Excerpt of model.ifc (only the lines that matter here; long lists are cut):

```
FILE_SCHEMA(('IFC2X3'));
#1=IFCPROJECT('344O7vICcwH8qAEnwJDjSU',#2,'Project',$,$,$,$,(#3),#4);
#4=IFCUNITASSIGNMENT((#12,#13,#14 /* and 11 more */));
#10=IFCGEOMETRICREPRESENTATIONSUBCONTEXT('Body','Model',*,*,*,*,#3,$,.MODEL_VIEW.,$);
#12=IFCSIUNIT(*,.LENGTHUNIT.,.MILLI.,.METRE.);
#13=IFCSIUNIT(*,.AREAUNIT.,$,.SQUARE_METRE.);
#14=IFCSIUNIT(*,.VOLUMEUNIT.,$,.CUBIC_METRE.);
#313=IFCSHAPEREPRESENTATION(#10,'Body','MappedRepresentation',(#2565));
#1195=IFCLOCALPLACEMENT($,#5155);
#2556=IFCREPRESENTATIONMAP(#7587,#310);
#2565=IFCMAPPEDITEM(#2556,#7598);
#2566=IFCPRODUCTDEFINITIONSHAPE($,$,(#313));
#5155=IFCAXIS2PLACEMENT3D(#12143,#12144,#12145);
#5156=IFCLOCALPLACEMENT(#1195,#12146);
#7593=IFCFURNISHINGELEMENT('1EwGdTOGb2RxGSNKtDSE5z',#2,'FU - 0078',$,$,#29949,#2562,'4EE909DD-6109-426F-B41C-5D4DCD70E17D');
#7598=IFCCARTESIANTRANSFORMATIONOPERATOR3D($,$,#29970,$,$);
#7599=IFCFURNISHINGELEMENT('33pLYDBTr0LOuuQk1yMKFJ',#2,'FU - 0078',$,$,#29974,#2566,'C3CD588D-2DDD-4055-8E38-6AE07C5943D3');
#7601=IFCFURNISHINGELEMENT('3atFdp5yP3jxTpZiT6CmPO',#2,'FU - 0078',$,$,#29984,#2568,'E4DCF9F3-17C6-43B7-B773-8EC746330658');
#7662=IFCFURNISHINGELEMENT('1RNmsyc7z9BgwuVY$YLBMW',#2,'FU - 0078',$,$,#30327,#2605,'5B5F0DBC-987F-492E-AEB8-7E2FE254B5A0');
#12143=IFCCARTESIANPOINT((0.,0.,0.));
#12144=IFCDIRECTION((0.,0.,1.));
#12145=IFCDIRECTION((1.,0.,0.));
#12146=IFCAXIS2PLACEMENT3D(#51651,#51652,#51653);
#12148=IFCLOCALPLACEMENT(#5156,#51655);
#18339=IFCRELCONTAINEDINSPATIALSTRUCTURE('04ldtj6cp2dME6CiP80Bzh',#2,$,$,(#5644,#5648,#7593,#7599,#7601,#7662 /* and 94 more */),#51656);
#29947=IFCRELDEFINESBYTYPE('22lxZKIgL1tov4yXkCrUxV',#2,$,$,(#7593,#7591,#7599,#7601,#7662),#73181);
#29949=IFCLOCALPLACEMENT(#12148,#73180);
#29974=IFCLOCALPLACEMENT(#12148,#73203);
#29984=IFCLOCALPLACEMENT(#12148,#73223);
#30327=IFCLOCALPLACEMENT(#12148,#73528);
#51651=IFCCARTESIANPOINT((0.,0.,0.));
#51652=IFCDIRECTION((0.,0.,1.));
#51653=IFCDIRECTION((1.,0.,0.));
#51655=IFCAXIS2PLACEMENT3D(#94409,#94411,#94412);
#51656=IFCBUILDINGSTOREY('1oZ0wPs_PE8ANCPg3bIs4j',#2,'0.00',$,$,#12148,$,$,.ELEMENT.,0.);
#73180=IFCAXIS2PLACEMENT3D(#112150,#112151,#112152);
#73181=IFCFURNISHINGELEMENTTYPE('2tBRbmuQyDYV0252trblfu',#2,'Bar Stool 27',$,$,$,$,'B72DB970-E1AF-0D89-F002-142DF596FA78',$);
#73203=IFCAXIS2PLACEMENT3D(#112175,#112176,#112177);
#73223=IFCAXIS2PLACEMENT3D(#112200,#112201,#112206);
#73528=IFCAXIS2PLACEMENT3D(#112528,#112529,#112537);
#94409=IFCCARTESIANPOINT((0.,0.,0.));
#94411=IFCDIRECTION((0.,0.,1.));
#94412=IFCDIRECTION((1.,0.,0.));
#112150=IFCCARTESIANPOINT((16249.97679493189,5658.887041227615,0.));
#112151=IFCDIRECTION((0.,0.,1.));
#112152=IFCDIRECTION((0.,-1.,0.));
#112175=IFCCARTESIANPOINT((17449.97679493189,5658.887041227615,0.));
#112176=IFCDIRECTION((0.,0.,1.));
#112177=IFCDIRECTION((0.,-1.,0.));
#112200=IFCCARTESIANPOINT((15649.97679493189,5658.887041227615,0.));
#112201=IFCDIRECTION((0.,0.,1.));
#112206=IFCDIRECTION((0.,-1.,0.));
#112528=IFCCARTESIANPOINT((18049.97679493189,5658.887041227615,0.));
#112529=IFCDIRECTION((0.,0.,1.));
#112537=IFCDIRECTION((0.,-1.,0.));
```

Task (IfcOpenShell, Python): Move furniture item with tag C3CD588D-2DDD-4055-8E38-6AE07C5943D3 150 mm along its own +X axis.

```python
import ifcopenshell
import ifcopenshell.api.geometry
import ifcopenshell.util.placement

model = ifcopenshell.open("model.ifc")

item = model.by_guid("33pLYDBTr0LOuuQk1yMKFJ")
matrix = ifcopenshell.util.placement.get_local_placement(item.ObjectPlacement)
matrix[:3, 3] += matrix[:3, 0] * 150.0
ifcopenshell.api.geometry.edit_object_placement(model, product=item, matrix=matrix, is_si=False)

print(ifcopenshell.util.placement.get_local_placement(item.ObjectPlacement).round(3) + 0.0)

model.write("model_edited.ifc")
```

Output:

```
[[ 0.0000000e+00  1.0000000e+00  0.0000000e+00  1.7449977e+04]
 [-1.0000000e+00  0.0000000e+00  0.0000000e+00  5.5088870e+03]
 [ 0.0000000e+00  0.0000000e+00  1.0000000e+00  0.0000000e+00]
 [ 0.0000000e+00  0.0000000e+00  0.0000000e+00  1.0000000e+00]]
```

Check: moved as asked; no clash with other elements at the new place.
